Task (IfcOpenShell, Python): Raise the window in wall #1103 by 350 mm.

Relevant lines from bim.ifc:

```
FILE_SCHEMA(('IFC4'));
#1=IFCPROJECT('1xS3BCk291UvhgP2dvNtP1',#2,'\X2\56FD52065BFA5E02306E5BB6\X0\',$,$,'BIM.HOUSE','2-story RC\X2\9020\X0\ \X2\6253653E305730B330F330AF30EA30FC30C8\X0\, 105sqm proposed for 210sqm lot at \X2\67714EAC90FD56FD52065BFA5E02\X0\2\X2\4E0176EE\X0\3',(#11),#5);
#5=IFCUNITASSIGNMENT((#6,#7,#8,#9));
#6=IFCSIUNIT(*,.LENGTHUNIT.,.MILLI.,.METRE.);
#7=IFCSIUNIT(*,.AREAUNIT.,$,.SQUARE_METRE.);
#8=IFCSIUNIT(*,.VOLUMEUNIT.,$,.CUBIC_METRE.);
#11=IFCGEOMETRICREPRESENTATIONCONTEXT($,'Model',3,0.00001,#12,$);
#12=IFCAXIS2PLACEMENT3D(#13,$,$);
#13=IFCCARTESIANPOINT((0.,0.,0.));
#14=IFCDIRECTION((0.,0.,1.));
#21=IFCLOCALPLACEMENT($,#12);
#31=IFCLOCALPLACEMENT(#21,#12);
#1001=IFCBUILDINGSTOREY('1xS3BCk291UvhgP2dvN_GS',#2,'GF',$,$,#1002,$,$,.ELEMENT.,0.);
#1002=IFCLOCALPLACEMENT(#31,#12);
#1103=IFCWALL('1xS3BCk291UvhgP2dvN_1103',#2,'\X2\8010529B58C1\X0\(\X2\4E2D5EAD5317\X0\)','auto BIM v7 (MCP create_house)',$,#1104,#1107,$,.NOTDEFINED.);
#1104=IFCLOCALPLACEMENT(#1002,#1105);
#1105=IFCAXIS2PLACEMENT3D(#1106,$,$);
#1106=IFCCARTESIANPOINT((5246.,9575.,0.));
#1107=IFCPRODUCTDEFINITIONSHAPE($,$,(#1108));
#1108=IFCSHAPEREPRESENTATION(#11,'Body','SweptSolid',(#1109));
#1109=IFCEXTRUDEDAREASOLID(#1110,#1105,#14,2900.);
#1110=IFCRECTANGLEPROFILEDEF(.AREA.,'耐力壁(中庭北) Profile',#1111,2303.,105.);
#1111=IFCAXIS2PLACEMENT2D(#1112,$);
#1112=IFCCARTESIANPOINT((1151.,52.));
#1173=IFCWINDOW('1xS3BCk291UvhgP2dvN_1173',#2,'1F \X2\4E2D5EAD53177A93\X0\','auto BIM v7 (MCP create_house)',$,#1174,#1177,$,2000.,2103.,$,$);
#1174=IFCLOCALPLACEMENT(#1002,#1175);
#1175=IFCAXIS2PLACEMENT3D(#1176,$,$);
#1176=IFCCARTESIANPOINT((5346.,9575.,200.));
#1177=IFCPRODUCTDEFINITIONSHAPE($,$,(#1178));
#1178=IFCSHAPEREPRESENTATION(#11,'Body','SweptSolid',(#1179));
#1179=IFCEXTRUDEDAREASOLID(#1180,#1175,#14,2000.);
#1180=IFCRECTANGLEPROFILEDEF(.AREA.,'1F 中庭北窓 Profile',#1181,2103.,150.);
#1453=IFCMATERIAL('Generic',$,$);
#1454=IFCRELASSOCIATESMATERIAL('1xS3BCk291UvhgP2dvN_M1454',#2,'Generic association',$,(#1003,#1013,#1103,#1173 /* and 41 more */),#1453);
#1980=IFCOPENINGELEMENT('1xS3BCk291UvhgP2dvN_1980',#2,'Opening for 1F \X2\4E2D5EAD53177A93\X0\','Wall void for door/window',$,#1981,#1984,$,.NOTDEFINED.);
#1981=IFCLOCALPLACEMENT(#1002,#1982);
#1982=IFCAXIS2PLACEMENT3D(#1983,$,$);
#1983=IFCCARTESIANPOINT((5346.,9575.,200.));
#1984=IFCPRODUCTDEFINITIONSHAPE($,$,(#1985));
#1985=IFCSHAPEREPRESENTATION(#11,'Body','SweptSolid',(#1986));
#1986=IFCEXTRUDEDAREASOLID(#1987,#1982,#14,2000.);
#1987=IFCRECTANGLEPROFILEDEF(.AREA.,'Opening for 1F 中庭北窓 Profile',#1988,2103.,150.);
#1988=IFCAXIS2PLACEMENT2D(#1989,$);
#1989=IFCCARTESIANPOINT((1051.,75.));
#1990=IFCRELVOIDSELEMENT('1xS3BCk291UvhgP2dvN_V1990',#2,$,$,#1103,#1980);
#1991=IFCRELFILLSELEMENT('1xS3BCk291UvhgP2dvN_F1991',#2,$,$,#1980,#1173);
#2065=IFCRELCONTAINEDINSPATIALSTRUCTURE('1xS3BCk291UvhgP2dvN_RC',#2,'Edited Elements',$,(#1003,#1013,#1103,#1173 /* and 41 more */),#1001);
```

```python
import numpy as np
import ifcopenshell
import ifcopenshell.api.geometry
import ifcopenshell.util.placement
import ifcopenshell.util.unit

model = ifcopenshell.open("bim.ifc")
unit_scale = ifcopenshell.util.unit.calculate_unit_scale(model)

window = model.by_guid("1xS3BCk291UvhgP2dvN_1173")
opening = window.FillsVoids[0].RelatingOpeningElement
dz = 350.0

shift = np.array([0.0, 0.0, dz])
# The window is not placed relative to its opening, so move both.
for product in (opening, window):
    matrix = ifcopenshell.util.placement.get_local_placement(product.ObjectPlacement)
    matrix[:3, 3] += shift
    ifcopenshell.api.geometry.edit_object_placement(model, product=product, matrix=matrix, is_si=False)

print(f"moved by {dz * unit_scale:+.3f} m")

model.write("bim_rev.ifc")
```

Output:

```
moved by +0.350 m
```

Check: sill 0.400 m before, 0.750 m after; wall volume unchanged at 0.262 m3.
